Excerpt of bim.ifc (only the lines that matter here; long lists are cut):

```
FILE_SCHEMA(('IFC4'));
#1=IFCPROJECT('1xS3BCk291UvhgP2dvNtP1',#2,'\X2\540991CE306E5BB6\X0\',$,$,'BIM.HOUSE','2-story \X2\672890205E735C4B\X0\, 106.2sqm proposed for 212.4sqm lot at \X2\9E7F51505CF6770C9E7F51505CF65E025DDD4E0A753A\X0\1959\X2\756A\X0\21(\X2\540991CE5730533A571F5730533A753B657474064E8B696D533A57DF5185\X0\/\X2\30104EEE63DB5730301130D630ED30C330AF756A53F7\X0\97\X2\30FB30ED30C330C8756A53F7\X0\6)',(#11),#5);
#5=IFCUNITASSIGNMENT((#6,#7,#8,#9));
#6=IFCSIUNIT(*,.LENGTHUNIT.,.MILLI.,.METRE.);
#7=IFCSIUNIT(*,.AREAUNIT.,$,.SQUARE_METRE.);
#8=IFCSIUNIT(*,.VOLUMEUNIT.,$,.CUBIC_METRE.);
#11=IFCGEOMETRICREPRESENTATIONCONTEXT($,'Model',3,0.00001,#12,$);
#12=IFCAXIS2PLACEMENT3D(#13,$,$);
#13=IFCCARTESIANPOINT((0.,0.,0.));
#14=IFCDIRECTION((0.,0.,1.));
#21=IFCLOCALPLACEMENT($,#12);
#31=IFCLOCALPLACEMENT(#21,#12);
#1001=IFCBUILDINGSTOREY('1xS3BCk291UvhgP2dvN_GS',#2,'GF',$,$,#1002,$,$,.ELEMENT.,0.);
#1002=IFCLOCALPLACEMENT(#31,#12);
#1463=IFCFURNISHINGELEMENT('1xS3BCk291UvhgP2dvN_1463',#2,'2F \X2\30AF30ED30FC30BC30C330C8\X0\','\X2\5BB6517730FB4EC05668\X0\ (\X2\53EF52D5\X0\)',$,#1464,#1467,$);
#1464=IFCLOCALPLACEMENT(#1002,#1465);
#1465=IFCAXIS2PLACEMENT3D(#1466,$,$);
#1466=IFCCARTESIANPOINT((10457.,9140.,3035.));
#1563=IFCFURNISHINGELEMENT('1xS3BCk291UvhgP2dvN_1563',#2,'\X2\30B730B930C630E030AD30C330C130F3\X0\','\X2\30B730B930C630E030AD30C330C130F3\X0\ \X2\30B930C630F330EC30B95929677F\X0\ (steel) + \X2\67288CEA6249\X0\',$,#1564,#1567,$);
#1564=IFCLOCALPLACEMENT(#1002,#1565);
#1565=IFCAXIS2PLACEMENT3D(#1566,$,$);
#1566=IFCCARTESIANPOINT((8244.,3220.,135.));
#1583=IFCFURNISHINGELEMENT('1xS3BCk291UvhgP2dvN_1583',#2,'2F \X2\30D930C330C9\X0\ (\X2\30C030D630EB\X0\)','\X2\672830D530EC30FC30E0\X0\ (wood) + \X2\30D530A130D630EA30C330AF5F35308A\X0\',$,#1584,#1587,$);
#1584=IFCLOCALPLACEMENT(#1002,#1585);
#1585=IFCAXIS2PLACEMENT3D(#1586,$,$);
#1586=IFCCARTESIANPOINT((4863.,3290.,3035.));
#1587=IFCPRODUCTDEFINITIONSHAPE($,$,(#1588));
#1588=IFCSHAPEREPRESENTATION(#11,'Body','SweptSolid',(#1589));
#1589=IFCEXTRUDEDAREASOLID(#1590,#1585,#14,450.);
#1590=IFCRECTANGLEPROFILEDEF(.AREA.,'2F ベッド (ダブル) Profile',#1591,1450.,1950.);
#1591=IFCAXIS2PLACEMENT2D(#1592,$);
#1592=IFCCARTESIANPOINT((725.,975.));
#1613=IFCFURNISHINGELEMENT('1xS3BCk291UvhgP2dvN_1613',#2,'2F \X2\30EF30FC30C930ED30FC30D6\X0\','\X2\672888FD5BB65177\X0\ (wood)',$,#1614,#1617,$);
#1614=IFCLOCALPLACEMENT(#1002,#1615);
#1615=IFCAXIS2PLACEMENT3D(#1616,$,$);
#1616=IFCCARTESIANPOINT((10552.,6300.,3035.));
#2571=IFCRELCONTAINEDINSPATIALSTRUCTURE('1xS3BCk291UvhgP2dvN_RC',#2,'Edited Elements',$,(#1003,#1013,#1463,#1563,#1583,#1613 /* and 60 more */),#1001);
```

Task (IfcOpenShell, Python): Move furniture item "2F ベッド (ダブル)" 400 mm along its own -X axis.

```python
import ifcopenshell
import ifcopenshell.api.geometry
import ifcopenshell.util.placement
import ifcopenshell.util.unit

model = ifcopenshell.open("bim.ifc")
unit_scale = ifcopenshell.util.unit.calculate_unit_scale(model)

item = model.by_guid("1xS3BCk291UvhgP2dvN_1583")
matrix = ifcopenshell.util.placement.get_local_placement(item.ObjectPlacement)
matrix[:3, 3] -= matrix[:3, 0] * 0.4 / unit_scale
ifcopenshell.api.geometry.edit_object_placement(model, product=item, matrix=matrix, is_si=False)

print(ifcopenshell.util.placement.get_local_placement(item.ObjectPlacement).round(3) + 0.0)

model.write("bim_rev.ifc")
```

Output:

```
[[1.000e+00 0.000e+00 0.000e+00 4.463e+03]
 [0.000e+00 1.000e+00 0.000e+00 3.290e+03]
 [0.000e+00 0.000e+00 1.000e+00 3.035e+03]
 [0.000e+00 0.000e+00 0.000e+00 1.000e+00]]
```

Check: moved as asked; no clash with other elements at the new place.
